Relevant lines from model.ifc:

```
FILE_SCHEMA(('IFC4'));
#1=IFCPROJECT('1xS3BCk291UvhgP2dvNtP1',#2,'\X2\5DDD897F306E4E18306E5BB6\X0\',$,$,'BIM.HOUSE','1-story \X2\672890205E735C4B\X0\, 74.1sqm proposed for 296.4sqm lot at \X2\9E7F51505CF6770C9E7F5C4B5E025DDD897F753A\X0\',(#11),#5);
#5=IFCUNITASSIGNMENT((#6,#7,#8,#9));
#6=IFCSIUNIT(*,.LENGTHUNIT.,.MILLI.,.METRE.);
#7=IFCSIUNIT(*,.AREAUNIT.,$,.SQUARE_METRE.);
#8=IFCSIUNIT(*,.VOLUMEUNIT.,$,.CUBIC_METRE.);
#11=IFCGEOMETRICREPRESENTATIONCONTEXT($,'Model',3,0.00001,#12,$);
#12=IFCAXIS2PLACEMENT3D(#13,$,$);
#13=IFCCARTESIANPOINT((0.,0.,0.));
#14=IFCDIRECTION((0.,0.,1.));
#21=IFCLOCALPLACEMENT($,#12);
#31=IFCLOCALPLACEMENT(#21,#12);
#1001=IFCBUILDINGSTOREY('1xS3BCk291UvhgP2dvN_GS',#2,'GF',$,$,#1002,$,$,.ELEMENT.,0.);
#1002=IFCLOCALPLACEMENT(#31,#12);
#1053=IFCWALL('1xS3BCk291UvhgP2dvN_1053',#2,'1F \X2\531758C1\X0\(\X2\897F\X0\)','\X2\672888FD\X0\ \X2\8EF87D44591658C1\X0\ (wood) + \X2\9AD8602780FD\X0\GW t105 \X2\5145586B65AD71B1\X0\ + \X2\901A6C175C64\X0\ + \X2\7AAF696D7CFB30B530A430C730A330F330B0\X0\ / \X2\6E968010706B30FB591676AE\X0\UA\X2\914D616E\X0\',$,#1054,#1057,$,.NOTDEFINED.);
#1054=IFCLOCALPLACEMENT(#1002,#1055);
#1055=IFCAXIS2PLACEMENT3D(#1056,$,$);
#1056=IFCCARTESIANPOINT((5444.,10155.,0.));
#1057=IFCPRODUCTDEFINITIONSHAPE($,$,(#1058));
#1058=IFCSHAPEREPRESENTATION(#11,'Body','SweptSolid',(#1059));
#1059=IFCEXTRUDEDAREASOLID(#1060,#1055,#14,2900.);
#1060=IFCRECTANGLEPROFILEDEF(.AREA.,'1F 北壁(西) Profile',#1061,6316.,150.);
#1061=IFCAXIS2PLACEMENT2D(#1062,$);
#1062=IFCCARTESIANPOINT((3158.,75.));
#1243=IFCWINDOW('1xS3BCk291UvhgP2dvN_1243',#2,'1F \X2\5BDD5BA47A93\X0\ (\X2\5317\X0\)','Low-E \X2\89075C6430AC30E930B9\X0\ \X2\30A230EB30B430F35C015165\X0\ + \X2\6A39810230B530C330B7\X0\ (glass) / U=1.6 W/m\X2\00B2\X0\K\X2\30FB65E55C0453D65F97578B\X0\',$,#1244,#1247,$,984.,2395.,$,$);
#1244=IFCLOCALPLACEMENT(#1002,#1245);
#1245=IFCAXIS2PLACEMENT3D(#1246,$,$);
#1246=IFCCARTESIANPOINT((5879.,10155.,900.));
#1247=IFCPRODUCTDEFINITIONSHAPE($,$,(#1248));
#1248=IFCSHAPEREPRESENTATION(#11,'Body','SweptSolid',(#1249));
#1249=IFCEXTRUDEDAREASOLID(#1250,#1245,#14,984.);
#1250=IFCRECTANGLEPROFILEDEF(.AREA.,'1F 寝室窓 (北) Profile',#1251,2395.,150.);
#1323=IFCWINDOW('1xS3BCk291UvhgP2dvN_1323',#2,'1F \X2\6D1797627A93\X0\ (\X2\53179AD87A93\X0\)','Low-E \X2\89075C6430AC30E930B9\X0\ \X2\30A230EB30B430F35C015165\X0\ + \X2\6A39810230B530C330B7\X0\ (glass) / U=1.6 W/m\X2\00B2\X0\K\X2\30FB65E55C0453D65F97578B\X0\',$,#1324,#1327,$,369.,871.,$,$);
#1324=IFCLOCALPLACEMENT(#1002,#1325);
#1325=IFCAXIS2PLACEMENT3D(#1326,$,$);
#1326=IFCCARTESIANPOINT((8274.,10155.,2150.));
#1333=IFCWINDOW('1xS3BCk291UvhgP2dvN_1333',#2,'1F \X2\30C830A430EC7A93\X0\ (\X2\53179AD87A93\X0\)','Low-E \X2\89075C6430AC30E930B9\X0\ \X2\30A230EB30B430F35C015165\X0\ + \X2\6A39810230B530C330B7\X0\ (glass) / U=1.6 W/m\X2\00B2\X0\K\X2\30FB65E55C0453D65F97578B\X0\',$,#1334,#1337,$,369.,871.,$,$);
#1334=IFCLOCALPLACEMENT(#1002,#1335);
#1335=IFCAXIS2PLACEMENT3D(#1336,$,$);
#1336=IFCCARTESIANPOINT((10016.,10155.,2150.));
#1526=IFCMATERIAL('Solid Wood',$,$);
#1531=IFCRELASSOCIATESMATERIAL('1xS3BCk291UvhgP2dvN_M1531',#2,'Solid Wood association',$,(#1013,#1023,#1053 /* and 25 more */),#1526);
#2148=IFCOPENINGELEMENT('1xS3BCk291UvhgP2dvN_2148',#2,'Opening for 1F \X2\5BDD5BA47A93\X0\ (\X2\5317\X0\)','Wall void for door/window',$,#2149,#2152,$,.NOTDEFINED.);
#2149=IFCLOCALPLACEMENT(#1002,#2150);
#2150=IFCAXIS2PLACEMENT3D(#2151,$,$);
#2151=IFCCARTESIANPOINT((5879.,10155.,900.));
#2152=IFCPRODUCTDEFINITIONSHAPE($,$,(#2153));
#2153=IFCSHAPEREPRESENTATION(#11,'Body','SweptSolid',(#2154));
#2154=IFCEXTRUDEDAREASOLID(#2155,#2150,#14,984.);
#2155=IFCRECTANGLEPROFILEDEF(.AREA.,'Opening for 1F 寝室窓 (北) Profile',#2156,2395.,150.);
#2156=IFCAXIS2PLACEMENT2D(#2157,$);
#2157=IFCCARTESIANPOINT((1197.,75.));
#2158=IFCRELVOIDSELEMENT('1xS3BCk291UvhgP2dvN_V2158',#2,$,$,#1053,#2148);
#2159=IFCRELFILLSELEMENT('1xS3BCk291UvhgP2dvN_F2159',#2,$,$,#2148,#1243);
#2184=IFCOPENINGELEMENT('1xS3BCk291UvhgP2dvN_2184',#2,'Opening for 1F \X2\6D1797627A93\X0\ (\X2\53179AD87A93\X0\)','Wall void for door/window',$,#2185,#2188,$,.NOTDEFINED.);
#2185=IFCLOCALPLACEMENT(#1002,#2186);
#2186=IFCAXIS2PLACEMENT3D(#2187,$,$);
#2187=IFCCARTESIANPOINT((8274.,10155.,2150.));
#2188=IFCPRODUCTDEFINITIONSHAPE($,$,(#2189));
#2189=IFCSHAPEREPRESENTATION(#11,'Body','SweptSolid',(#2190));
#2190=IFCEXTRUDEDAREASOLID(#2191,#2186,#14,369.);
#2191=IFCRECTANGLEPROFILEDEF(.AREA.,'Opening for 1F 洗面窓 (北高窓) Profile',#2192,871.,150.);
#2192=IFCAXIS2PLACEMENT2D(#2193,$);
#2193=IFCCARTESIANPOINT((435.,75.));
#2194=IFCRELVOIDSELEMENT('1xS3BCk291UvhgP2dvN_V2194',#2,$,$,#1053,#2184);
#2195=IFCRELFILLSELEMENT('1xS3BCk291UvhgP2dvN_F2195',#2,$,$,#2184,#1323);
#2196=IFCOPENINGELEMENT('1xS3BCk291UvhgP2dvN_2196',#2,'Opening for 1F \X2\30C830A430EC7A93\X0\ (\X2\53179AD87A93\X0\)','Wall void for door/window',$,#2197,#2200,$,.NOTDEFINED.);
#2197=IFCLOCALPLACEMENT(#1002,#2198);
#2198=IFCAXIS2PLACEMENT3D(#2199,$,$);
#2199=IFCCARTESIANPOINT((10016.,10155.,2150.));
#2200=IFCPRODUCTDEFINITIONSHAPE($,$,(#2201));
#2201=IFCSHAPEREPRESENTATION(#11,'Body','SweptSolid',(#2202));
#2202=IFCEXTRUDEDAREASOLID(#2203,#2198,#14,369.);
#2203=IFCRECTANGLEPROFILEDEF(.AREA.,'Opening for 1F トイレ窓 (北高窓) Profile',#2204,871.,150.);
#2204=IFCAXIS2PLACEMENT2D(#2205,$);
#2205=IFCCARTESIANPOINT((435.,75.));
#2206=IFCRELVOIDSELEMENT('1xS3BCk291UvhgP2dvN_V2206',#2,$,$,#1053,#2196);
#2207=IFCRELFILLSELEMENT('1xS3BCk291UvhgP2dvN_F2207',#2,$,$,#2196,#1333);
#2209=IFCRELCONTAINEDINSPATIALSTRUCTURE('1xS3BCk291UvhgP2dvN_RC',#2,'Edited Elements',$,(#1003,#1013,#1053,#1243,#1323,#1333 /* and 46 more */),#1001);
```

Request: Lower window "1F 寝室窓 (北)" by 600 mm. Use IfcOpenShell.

```python
import numpy as np
import ifcopenshell
import ifcopenshell.api.geometry
import ifcopenshell.util.placement
import ifcopenshell.util.unit

model = ifcopenshell.open("model.ifc")
unit_scale = ifcopenshell.util.unit.calculate_unit_scale(model)

window = model.by_guid("1xS3BCk291UvhgP2dvN_1243")
opening = window.FillsVoids[0].RelatingOpeningElement
dz = -0.6 / unit_scale

shift = np.array([0.0, 0.0, dz])
# The window is not placed relative to its opening, so move both.
for product in (opening, window):
    matrix = ifcopenshell.util.placement.get_local_placement(product.ObjectPlacement)
    matrix[:3, 3] += shift
    ifcopenshell.api.geometry.edit_object_placement(model, product=product, matrix=matrix, is_si=False)

print(f"moved by {dz * unit_scale:+.3f} m")

model.write("model_updated.ifc")
```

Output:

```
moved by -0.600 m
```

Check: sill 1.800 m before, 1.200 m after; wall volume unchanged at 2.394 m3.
